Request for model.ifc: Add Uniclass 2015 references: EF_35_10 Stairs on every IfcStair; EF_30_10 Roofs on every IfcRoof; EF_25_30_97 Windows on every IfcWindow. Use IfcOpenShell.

First a look at what the model holds.

```python
import ifcopenshell

model = ifcopenshell.open("model.ifc")
print(model.schema)
print("classifications:", [c.Name for c in model.by_type("IfcClassification")])
for ifc_class in ("IfcDoor", "IfcRoof", "IfcStair", "IfcWall", "IfcWindow"):
    print(ifc_class, len(model.by_type(ifc_class)))
```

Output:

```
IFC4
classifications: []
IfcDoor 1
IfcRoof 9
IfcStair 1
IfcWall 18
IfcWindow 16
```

```python
import ifcopenshell
import ifcopenshell.api.classification

model = ifcopenshell.open("model.ifc")

system = ifcopenshell.api.classification.add_classification(model, classification="Uniclass 2015")

codes = {
    "IfcStair": ("EF_35_10", "Stairs"),
    "IfcRoof": ("EF_30_10", "Roofs"),
    "IfcWindow": ("EF_25_30_97", "Windows"),
}
for ifc_class, (code, name) in codes.items():
    products = model.by_type(ifc_class)
    ifcopenshell.api.classification.add_reference(
        model, products=products, classification=system, identification=code, name=name
    )
    print(code, len(products))

model.write("model_updated.ifc")
```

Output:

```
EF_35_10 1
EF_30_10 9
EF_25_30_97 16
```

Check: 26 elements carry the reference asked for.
